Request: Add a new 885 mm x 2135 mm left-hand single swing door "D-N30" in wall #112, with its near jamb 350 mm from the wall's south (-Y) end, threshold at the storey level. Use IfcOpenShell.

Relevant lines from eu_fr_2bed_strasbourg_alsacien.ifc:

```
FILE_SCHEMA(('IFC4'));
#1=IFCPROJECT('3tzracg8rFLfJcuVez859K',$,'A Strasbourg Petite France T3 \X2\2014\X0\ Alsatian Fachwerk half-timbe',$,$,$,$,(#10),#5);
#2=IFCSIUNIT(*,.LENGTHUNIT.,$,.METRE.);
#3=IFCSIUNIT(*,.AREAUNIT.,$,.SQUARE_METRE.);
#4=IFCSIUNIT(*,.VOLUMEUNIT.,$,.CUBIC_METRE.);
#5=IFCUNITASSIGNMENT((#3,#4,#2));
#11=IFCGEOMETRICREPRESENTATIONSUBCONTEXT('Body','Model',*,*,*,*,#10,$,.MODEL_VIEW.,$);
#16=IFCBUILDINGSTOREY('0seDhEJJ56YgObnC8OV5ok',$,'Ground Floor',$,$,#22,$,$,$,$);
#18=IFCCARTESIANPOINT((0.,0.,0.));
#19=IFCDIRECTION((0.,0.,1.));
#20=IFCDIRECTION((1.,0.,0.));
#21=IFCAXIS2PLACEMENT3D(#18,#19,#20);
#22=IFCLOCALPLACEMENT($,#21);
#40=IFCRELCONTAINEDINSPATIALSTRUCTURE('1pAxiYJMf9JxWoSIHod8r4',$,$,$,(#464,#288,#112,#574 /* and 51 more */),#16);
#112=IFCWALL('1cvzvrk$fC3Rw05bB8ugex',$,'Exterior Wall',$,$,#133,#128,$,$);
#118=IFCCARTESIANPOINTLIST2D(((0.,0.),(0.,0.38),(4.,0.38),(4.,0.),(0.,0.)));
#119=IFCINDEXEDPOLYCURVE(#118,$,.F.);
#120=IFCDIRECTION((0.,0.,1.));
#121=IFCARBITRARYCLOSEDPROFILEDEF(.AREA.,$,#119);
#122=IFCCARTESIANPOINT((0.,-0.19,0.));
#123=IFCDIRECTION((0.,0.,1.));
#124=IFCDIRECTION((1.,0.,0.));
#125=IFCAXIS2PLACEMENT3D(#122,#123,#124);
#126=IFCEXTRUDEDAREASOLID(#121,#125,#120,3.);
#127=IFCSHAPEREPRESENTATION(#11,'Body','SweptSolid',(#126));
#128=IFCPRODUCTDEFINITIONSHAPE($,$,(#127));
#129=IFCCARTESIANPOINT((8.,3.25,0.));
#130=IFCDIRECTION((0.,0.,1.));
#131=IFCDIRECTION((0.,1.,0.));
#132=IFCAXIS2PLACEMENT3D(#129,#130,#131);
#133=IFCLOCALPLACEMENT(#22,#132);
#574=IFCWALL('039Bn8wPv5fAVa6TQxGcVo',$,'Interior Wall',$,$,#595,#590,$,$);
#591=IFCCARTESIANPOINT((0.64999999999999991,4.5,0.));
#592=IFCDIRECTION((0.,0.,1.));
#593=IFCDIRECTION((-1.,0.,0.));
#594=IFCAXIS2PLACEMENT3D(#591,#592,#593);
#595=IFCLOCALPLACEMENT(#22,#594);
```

```python
import numpy as np
import ifcopenshell
import ifcopenshell.api.feature
import ifcopenshell.api.geometry
import ifcopenshell.api.root
import ifcopenshell.api.spatial
import ifcopenshell.geom
import ifcopenshell.util.element
import ifcopenshell.util.placement
import ifcopenshell.util.representation
import ifcopenshell.util.shape
import ifcopenshell.util.unit

model = ifcopenshell.open("eu_fr_2bed_strasbourg_alsacien.ifc")
unit_scale = ifcopenshell.util.unit.calculate_unit_scale(model)
settings = ifcopenshell.geom.settings()


def volume(element):
    """Net volume in cubic metres, openings subtracted."""
    shape = ifcopenshell.geom.create_shape(settings, element)
    return ifcopenshell.util.shape.get_volume(shape.geometry)


wall = model.by_id(112)
storey = ifcopenshell.util.element.get_container(wall, ifc_class="IfcBuildingStorey")
context = ifcopenshell.util.representation.get_context(model, "Model", "Body", "MODEL_VIEW")
before = volume(wall)

width, height, from_end, sill = 0.885, 2.135, 0.35, 0.0  # metres

# The wall runs along its own X axis, and the end named is its -X end.
wall_shape = ifcopenshell.geom.create_shape(settings, wall)
x, y, z = ifcopenshell.util.shape.get_vertices(wall_shape.geometry).T
start = x.min() + from_end
face, thickness = float(y.min()), float(y.max() - y.min())
wall_matrix = ifcopenshell.util.placement.get_local_placement(wall.ObjectPlacement)
level = ifcopenshell.util.placement.get_local_placement(storey.ObjectPlacement)[2, 3]


def in_wall(x, y):
    """Placement at x, y metres in the wall's axes, at sill height."""
    matrix = wall_matrix.copy()
    matrix[:, 3] = wall_matrix @ np.array([x / unit_scale, y / unit_scale, 0.0, 1.0])
    matrix[2, 3] = level + sill / unit_scale
    return matrix


# Opening: a box that overshoots both wall faces by 50 mm.
opening = ifcopenshell.api.root.create_entity(model, ifc_class="IfcOpeningElement", predefined_type="OPENING")
box = ifcopenshell.api.geometry.add_wall_representation(
    model, context=context, length=width, height=height, thickness=thickness + 0.1
)
ifcopenshell.api.geometry.assign_representation(model, product=opening, representation=box)
ifcopenshell.api.geometry.edit_object_placement(model, product=opening, matrix=in_wall(start, face - 0.05), is_si=False)
ifcopenshell.api.feature.add_feature(model, feature=opening, element=wall)

door = ifcopenshell.api.root.create_entity(model, ifc_class="IfcDoor", name="D-N30", predefined_type="DOOR")
door.OverallWidth, door.OverallHeight = width / unit_scale, height / unit_scale
door.OperationType = "SINGLE_SWING_LEFT"
body = ifcopenshell.api.geometry.add_door_representation(
    model,
    context=context,
    overall_width=door.OverallWidth,
    overall_height=door.OverallHeight,
    operation_type="SINGLE_SWING_LEFT",
    lining_properties={"LiningDepth": thickness / unit_scale, "ThresholdDepth": thickness / unit_scale},
)
ifcopenshell.api.geometry.assign_representation(model, product=door, representation=body)
ifcopenshell.api.spatial.assign_container(model, products=[door], relating_structure=storey)
ifcopenshell.api.feature.add_filling(model, opening=opening, element=door)

# The lining spans the wall, so the door starts at the wall face.
ifcopenshell.api.geometry.edit_object_placement(model, product=door, matrix=in_wall(start, face), is_si=False)

after = volume(wall)

print(f"wall volume {before:.3f} -> {after:.3f} m3")

model.write("eu_fr_2bed_strasbourg_alsacien_rev.ifc")
```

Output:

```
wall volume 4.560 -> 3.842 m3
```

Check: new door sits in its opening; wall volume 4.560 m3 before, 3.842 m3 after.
